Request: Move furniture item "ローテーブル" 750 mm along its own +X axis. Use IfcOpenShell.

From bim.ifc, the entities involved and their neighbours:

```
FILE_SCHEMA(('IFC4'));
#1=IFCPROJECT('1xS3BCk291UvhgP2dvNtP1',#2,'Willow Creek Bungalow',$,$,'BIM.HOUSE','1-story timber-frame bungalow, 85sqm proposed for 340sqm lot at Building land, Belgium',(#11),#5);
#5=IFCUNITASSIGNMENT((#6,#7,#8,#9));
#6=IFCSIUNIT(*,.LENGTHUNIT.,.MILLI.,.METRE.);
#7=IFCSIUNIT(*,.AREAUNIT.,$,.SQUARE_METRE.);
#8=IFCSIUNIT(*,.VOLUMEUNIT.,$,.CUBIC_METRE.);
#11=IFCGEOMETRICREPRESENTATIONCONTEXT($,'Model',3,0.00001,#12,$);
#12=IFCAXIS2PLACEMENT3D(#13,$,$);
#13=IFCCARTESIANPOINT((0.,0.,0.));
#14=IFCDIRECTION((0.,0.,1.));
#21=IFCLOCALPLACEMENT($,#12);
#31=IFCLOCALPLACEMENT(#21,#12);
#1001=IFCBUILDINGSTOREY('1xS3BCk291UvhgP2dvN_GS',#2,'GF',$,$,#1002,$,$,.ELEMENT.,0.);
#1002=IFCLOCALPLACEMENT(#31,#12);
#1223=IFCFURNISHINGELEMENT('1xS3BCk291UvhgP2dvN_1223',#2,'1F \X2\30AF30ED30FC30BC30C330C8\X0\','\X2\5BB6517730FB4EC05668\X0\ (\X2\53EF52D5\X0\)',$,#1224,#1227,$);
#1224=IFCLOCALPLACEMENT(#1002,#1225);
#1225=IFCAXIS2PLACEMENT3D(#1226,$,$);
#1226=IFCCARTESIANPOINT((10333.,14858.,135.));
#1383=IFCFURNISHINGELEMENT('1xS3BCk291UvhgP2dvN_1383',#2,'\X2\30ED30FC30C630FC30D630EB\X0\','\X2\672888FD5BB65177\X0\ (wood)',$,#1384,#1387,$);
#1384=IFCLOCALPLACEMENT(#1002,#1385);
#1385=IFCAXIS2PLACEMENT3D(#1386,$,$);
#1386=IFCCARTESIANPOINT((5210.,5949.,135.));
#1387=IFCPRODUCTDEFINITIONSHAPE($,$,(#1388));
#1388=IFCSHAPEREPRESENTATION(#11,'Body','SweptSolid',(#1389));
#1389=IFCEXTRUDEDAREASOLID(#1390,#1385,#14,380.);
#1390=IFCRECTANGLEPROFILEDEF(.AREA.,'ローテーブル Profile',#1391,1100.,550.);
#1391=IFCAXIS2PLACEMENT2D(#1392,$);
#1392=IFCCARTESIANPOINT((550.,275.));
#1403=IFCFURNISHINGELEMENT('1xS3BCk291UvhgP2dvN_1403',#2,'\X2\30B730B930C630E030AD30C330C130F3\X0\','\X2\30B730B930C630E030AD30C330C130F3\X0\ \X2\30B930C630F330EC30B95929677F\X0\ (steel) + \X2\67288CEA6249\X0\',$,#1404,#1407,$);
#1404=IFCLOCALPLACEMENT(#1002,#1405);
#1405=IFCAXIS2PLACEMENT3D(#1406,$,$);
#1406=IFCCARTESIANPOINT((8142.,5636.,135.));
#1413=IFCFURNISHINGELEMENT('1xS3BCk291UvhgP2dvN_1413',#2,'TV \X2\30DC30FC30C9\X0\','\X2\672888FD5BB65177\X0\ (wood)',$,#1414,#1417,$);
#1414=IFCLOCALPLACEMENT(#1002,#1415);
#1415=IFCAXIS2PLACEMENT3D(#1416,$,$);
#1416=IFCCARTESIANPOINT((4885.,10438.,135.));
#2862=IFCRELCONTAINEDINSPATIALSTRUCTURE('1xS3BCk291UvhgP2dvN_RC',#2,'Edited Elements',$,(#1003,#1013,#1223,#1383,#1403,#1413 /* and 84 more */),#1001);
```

```python
import ifcopenshell
import ifcopenshell.api.geometry
import ifcopenshell.util.placement
import ifcopenshell.util.unit

model = ifcopenshell.open("bim.ifc")
unit_scale = ifcopenshell.util.unit.calculate_unit_scale(model)

item = model.by_guid("1xS3BCk291UvhgP2dvN_1383")
matrix = ifcopenshell.util.placement.get_local_placement(item.ObjectPlacement)
matrix[:3, 3] += matrix[:3, 0] * 0.75 / unit_scale
ifcopenshell.api.geometry.edit_object_placement(model, product=item, matrix=matrix, is_si=False)

print(ifcopenshell.util.placement.get_local_placement(item.ObjectPlacement).round(3) + 0.0)

model.write("bim_edited.ifc")
```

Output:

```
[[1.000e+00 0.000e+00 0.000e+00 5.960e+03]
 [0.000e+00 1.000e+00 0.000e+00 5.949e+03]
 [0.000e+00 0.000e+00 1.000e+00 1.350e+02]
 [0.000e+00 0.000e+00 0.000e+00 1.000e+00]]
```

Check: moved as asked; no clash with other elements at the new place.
